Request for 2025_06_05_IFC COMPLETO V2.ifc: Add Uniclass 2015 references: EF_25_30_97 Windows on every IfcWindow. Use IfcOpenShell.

First a look at what the model holds.

```python
import ifcopenshell

model = ifcopenshell.open("2025_06_05_IFC COMPLETO V2.ifc")
print(model.schema)
print("classifications:", [c.Name for c in model.by_type("IfcClassification")])
for ifc_class in ("IfcDoor", "IfcRoof", "IfcStair", "IfcWall", "IfcWindow"):
    print(ifc_class, len(model.by_type(ifc_class)))
```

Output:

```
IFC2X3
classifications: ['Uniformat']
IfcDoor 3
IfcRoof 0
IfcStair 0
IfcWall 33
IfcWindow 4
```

```python
import ifcopenshell
import ifcopenshell.api.classification

model = ifcopenshell.open("2025_06_05_IFC COMPLETO V2.ifc")

# IFC2X3 requires Source and Edition and has no link from the project to the system.
system = model.create_entity("IfcClassification", Source="NBS", Edition="2015", Name="Uniclass 2015")

codes = {
    "IfcWindow": ("EF_25_30_97", "Windows"),
}
for ifc_class, (code, name) in codes.items():
    products = model.by_type(ifc_class)
    ifcopenshell.api.classification.add_reference(
        model, products=products, classification=system, identification=code, name=name
    )
    print(code, len(products))

model.write("2025_06_05_IFC COMPLETO V2_edited.ifc")
```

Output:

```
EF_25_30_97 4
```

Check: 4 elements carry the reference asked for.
